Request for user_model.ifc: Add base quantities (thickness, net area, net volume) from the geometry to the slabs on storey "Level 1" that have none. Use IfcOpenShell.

First a look at what the model holds.

```python
import ifcopenshell
import ifcopenshell.util.element
import ifcopenshell.util.unit

model = ifcopenshell.open("user_model.ifc")
print(model.schema)
for unit_type in ("LENGTHUNIT", "AREAUNIT", "VOLUMEUNIT"):
    print(unit_type, ifcopenshell.util.unit.calculate_unit_scale(model, unit_type))
storey = next(s for s in model.by_type("IfcBuildingStorey") if s.Name == "Level 1")
slabs = [e for e in ifcopenshell.util.element.get_decomposition(storey) if e.is_a("IfcSlab")]
for e in sorted(slabs, key=lambda e: e.id()):
    print(e.id(), e.is_a(), e.Name, list(ifcopenshell.util.element.get_psets(e, qtos_only=True)), sep=" | ")
```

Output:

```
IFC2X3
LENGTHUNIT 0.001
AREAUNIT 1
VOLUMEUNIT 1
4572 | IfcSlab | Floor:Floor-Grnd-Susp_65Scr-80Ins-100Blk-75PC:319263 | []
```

```python
import ifcopenshell
import ifcopenshell.api.pset
import ifcopenshell.geom
import ifcopenshell.util.element
import ifcopenshell.util.shape
import ifcopenshell.util.unit

model = ifcopenshell.open("user_model.ifc")
unit_scale = ifcopenshell.util.unit.calculate_unit_scale(model)
area_scale = ifcopenshell.util.unit.calculate_unit_scale(model, "AREAUNIT")
volume_scale = ifcopenshell.util.unit.calculate_unit_scale(model, "VOLUMEUNIT")
settings = ifcopenshell.geom.settings()

storey = next(s for s in model.by_type("IfcBuildingStorey") if s.Name == "Level 1")
slabs = [e for e in ifcopenshell.util.element.get_decomposition(storey) if e.is_a("IfcSlab")]

for e in sorted(slabs, key=lambda e: e.id()):
    if ifcopenshell.util.element.get_psets(e, qtos_only=True, should_inherit=False):
        continue
    # Geometry comes back in metres, in the element's own axes.
    shape = ifcopenshell.geom.create_shape(settings, e)
    values = {
        "Width": ifcopenshell.util.shape.get_z(shape.geometry) / unit_scale,
        "NetArea": ifcopenshell.util.shape.get_footprint_area(shape.geometry) / area_scale,
        "NetVolume": ifcopenshell.util.shape.get_volume(shape.geometry) / volume_scale,
    }
    qto = ifcopenshell.api.pset.add_qto(model, product=e, name="BaseQuantities")
    ifcopenshell.api.pset.edit_qto(model, qto=qto, properties=values)
    print(e.id(), {k: round(v, 3) for k, v in values.items()})

model.write("user_model_rev.ifc")
```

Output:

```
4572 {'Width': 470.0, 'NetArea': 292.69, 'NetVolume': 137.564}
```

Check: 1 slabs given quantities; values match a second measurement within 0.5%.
